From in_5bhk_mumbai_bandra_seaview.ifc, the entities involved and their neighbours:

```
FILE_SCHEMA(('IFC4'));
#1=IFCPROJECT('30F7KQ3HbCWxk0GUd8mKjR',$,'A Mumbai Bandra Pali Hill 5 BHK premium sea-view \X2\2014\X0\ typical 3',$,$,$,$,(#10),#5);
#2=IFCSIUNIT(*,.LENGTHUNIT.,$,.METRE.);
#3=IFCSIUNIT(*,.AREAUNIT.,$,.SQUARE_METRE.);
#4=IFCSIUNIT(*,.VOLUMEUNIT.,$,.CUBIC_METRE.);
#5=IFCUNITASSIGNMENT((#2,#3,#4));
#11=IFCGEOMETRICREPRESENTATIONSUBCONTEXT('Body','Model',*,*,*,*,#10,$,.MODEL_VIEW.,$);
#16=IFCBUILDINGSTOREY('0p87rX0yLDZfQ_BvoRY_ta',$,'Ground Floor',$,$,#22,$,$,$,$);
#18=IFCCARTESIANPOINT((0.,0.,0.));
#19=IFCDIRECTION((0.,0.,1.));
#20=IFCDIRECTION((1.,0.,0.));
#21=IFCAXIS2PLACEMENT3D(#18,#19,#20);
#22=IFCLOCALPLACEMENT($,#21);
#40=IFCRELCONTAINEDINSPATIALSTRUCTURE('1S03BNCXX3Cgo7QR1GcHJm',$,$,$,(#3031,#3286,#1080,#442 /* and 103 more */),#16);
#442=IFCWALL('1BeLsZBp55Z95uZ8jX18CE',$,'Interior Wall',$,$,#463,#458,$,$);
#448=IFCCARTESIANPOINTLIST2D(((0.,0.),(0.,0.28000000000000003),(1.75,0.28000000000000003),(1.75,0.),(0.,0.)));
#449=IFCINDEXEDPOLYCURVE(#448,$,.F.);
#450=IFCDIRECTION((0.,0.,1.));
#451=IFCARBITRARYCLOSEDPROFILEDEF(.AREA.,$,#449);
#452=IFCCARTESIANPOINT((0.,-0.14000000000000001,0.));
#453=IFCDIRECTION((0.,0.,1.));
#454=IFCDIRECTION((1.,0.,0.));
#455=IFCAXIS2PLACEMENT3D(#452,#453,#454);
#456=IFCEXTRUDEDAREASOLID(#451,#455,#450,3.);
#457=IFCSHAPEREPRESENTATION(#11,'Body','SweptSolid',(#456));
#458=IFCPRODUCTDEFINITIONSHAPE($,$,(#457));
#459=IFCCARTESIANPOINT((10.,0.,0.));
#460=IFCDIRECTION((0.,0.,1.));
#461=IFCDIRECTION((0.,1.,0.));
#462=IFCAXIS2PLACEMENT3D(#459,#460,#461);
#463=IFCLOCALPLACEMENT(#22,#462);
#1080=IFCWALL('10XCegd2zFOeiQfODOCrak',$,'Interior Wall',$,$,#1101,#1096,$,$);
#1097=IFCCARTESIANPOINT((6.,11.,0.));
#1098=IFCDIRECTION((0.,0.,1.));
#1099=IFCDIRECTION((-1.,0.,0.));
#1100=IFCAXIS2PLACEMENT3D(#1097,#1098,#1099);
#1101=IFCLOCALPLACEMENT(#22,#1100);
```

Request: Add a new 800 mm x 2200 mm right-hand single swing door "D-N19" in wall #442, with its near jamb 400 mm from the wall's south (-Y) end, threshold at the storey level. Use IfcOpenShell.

```python
import numpy as np
import ifcopenshell
import ifcopenshell.api.feature
import ifcopenshell.api.geometry
import ifcopenshell.api.root
import ifcopenshell.api.spatial
import ifcopenshell.geom
import ifcopenshell.util.element
import ifcopenshell.util.placement
import ifcopenshell.util.representation
import ifcopenshell.util.shape
import ifcopenshell.util.unit

model = ifcopenshell.open("in_5bhk_mumbai_bandra_seaview.ifc")
unit_scale = ifcopenshell.util.unit.calculate_unit_scale(model)
settings = ifcopenshell.geom.settings()


def volume(element):
    """Net volume in cubic metres, openings subtracted."""
    shape = ifcopenshell.geom.create_shape(settings, element)
    return ifcopenshell.util.shape.get_volume(shape.geometry)


wall = model.by_guid("1BeLsZBp55Z95uZ8jX18CE")
storey = ifcopenshell.util.element.get_container(wall, ifc_class="IfcBuildingStorey")
context = ifcopenshell.util.representation.get_context(model, "Model", "Body", "MODEL_VIEW")
before = volume(wall)

width, height, from_end, sill = 0.8, 2.2, 0.4, 0.0  # metres

# The wall runs along its own X axis, and the end named is its -X end.
wall_shape = ifcopenshell.geom.create_shape(settings, wall)
x, y, z = ifcopenshell.util.shape.get_vertices(wall_shape.geometry).T
start = x.min() + from_end
face, thickness = float(y.min()), float(y.max() - y.min())
wall_matrix = ifcopenshell.util.placement.get_local_placement(wall.ObjectPlacement)
level = ifcopenshell.util.placement.get_local_placement(storey.ObjectPlacement)[2, 3]


def in_wall(x, y):
    """Placement at x, y metres in the wall's axes, at sill height."""
    matrix = wall_matrix.copy()
    matrix[:, 3] = wall_matrix @ np.array([x / unit_scale, y / unit_scale, 0.0, 1.0])
    matrix[2, 3] = level + sill / unit_scale
    return matrix


# Opening: a box that overshoots both wall faces by 50 mm.
opening = ifcopenshell.api.root.create_entity(model, ifc_class="IfcOpeningElement", predefined_type="OPENING")
box = ifcopenshell.api.geometry.add_wall_representation(
    model, context=context, length=width, height=height, thickness=thickness + 0.1
)
ifcopenshell.api.geometry.assign_representation(model, product=opening, representation=box)
ifcopenshell.api.geometry.edit_object_placement(model, product=opening, matrix=in_wall(start, face - 0.05), is_si=False)
ifcopenshell.api.feature.add_feature(model, feature=opening, element=wall)

door = ifcopenshell.api.root.create_entity(model, ifc_class="IfcDoor", name="D-N19", predefined_type="DOOR")
door.OverallWidth, door.OverallHeight = width / unit_scale, height / unit_scale
door.OperationType = "SINGLE_SWING_RIGHT"
body = ifcopenshell.api.geometry.add_door_representation(
    model,
    context=context,
    overall_width=door.OverallWidth,
    overall_height=door.OverallHeight,
    operation_type="SINGLE_SWING_RIGHT",
    lining_properties={"LiningDepth": thickness / unit_scale, "ThresholdDepth": thickness / unit_scale},
)
ifcopenshell.api.geometry.assign_representation(model, product=door, representation=body)
ifcopenshell.api.spatial.assign_container(model, products=[door], relating_structure=storey)
ifcopenshell.api.feature.add_filling(model, opening=opening, element=door)

# The lining spans the wall, so the door starts at the wall face.
ifcopenshell.api.geometry.edit_object_placement(model, product=door, matrix=in_wall(start, face), is_si=False)

after = volume(wall)

print(f"wall volume {before:.3f} -> {after:.3f} m3")

model.write("in_5bhk_mumbai_bandra_seaview_edited.ifc")
```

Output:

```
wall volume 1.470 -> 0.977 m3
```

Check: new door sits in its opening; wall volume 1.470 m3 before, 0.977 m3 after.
